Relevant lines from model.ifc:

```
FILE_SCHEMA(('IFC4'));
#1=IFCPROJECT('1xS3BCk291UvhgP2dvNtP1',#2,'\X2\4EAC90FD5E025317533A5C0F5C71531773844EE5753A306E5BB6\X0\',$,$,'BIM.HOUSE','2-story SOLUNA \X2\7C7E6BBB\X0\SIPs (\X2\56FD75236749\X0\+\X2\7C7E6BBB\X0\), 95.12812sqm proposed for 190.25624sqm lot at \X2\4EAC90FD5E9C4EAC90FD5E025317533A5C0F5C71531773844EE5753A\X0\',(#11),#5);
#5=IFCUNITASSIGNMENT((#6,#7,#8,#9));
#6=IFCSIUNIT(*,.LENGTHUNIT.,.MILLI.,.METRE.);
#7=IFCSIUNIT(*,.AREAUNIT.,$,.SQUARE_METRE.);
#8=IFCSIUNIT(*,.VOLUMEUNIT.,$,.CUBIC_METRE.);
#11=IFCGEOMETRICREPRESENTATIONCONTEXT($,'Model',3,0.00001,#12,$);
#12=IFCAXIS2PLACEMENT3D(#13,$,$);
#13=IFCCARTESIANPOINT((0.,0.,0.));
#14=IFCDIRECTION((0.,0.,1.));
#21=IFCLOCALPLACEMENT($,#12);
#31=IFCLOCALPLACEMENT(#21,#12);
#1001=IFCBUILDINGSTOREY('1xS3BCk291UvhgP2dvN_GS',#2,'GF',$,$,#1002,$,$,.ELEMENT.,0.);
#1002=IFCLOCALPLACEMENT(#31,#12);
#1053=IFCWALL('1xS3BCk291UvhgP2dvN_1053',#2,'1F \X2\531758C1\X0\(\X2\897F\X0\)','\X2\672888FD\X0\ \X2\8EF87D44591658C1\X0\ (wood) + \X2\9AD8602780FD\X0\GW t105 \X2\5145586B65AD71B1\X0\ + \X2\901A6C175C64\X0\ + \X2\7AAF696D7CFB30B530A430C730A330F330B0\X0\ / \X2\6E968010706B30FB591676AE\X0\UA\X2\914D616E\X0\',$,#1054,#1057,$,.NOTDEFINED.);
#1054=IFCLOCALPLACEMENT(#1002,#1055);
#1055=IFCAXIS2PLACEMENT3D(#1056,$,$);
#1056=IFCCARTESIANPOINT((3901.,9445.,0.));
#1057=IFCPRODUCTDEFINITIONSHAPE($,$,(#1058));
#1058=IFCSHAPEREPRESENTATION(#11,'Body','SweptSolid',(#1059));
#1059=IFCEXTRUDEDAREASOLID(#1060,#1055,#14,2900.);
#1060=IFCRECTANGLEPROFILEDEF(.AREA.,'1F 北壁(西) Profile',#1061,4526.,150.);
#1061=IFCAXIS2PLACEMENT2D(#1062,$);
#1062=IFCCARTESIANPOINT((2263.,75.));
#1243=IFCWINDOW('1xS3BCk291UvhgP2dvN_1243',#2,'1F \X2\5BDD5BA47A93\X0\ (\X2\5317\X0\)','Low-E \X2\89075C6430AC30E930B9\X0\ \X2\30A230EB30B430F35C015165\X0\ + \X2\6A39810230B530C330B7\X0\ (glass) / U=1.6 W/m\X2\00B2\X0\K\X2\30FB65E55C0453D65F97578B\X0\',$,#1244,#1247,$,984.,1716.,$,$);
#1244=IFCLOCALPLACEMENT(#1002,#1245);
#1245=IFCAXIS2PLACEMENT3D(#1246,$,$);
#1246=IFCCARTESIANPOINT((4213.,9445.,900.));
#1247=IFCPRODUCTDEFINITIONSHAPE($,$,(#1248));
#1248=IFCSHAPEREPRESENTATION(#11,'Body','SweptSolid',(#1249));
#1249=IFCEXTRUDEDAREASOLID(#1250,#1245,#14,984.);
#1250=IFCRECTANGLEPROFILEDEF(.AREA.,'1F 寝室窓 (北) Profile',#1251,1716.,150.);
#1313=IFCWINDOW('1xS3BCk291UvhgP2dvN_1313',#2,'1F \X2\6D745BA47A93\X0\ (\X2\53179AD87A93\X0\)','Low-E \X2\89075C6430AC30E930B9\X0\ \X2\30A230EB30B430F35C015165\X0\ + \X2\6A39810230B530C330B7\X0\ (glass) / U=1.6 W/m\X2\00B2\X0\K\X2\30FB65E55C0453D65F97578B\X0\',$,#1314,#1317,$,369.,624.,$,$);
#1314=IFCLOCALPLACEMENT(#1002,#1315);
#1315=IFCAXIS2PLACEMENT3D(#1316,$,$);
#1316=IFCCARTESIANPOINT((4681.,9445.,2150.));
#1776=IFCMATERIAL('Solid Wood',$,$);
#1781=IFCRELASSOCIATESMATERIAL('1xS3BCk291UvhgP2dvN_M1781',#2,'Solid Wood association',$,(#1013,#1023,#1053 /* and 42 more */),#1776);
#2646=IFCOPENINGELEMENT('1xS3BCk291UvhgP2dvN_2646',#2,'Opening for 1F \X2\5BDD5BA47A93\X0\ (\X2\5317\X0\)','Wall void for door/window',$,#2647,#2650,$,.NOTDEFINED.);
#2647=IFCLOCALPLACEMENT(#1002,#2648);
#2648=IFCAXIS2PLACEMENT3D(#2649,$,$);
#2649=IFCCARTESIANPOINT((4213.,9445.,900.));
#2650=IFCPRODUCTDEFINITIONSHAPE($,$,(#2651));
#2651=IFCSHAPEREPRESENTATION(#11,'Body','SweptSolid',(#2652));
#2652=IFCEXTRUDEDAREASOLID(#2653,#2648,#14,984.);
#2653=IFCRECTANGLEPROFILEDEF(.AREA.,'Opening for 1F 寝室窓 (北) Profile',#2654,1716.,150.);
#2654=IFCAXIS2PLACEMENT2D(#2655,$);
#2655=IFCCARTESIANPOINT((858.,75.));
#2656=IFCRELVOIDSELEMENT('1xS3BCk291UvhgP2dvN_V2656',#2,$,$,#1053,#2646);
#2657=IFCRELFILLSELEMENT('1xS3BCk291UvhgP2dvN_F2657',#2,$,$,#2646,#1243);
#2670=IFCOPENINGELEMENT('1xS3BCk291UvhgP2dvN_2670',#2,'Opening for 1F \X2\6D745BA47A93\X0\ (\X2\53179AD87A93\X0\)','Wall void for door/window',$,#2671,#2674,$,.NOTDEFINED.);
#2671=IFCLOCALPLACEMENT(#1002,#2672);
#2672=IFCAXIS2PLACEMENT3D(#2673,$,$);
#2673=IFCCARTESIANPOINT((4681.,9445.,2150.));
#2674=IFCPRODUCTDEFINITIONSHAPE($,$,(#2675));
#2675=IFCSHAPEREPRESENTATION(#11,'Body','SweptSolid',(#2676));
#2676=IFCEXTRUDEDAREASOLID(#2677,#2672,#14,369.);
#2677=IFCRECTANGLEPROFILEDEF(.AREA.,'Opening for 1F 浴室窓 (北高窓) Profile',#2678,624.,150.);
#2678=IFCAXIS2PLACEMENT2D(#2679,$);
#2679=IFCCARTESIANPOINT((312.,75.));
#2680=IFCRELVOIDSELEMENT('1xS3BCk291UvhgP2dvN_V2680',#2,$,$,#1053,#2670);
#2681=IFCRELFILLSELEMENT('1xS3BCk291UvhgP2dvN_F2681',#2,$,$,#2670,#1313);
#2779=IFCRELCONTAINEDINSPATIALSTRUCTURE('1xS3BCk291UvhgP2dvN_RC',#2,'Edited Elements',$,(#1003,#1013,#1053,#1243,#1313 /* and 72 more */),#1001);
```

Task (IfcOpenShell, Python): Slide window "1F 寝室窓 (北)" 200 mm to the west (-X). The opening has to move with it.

```python
import ifcopenshell
import ifcopenshell.api.geometry
import ifcopenshell.util.placement
import ifcopenshell.util.unit

model = ifcopenshell.open("model.ifc")
unit_scale = ifcopenshell.util.unit.calculate_unit_scale(model)

window = model.by_guid("1xS3BCk291UvhgP2dvN_1243")
opening = window.FillsVoids[0].RelatingOpeningElement
wall = opening.VoidsElements[0].RelatingBuildingElement

wall_matrix = ifcopenshell.util.placement.get_local_placement(wall.ObjectPlacement)
shift = wall_matrix[:3, 0] * -0.2 / unit_scale
before = ifcopenshell.util.placement.get_local_placement(window.ObjectPlacement)[:3, 3].copy()

# The window is not placed relative to its opening, so move both.
for product in (opening, window):
    matrix = ifcopenshell.util.placement.get_local_placement(product.ObjectPlacement)
    matrix[:3, 3] += shift
    ifcopenshell.api.geometry.edit_object_placement(model, product=product, matrix=matrix, is_si=False)

after = ifcopenshell.util.placement.get_local_placement(window.ObjectPlacement)[:3, 3]
print("window moved by", (after - before).round(3) + 0.0)

model.write("model_v2.ifc")
```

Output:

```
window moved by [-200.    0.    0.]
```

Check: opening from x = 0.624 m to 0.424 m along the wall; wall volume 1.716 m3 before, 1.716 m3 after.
